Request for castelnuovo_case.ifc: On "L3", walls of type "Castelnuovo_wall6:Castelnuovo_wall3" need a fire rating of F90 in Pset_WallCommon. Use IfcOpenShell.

First a look at what the model holds.

```python
import ifcopenshell
import ifcopenshell.util.element

model = ifcopenshell.open("castelnuovo_case.ifc")
print(model.schema)
storey = next(s for s in model.by_type("IfcBuildingStorey") if s.Name == "L3")
walls = [e for e in ifcopenshell.util.element.get_decomposition(storey) if e.is_a("IfcWall")]
seen = {}
for e in walls:
    element_type = ifcopenshell.util.element.get_type(e)
    key = (element_type.Name if element_type != e and element_type else None, ifcopenshell.util.element.get_pset(e, "Pset_WallCommon", "FireRating"))
    seen[key] = seen.get(key, 0) + 1
for (name, value), count in sorted(seen.items(), key=str):
    print(count, "x", name, "|", value)
```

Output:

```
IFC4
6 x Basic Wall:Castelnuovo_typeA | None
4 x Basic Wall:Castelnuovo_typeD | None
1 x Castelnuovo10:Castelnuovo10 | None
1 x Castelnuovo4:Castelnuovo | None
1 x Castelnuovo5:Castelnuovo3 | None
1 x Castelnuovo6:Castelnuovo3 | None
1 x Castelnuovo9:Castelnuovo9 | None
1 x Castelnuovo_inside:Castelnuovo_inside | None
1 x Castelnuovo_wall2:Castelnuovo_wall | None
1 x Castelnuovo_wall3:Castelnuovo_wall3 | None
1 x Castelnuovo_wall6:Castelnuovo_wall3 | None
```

```python
import ifcopenshell
import ifcopenshell.api.pset
import ifcopenshell.util.element

model = ifcopenshell.open("castelnuovo_case.ifc")

storey = next(s for s in model.by_type("IfcBuildingStorey") if s.Name == "L3")
walls = [e for e in ifcopenshell.util.element.get_decomposition(storey) if e.is_a("IfcWall")]

count = 0
for e in walls:
    element_type = ifcopenshell.util.element.get_type(e)
    if element_type in (None, e) or element_type.Name != "Castelnuovo_wall6:Castelnuovo_wall3":
        continue
    # add_pset returns the element's existing set when there is one.
    pset = ifcopenshell.api.pset.add_pset(model, product=e, name="Pset_WallCommon")
    ifcopenshell.api.pset.edit_pset(model, pset=pset, properties={"FireRating": "F90"})
    count += 1

print(count, "walls updated")

model.write("castelnuovo_case_v2.ifc")
```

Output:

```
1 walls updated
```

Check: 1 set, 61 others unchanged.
